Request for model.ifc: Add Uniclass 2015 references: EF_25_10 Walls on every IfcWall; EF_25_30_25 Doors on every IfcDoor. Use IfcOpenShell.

First a look at what the model holds.

```python
import ifcopenshell

model = ifcopenshell.open("model.ifc")
print(model.schema)
print("classifications:", [c.Name for c in model.by_type("IfcClassification")])
for ifc_class in ("IfcDoor", "IfcRoof", "IfcStair", "IfcWall", "IfcWindow"):
    print(ifc_class, len(model.by_type(ifc_class)))
```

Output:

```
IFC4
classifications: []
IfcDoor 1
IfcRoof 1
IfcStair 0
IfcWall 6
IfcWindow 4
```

```python
import ifcopenshell
import ifcopenshell.api.classification

model = ifcopenshell.open("model.ifc")

system = ifcopenshell.api.classification.add_classification(model, classification="Uniclass 2015")

codes = {
    "IfcWall": ("EF_25_10", "Walls"),
    "IfcDoor": ("EF_25_30_25", "Doors"),
}
for ifc_class, (code, name) in codes.items():
    products = model.by_type(ifc_class)
    ifcopenshell.api.classification.add_reference(
        model, products=products, classification=system, identification=code, name=name
    )
    print(code, len(products))

model.write("model-out.ifc")
```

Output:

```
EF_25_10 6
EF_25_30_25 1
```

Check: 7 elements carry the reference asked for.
